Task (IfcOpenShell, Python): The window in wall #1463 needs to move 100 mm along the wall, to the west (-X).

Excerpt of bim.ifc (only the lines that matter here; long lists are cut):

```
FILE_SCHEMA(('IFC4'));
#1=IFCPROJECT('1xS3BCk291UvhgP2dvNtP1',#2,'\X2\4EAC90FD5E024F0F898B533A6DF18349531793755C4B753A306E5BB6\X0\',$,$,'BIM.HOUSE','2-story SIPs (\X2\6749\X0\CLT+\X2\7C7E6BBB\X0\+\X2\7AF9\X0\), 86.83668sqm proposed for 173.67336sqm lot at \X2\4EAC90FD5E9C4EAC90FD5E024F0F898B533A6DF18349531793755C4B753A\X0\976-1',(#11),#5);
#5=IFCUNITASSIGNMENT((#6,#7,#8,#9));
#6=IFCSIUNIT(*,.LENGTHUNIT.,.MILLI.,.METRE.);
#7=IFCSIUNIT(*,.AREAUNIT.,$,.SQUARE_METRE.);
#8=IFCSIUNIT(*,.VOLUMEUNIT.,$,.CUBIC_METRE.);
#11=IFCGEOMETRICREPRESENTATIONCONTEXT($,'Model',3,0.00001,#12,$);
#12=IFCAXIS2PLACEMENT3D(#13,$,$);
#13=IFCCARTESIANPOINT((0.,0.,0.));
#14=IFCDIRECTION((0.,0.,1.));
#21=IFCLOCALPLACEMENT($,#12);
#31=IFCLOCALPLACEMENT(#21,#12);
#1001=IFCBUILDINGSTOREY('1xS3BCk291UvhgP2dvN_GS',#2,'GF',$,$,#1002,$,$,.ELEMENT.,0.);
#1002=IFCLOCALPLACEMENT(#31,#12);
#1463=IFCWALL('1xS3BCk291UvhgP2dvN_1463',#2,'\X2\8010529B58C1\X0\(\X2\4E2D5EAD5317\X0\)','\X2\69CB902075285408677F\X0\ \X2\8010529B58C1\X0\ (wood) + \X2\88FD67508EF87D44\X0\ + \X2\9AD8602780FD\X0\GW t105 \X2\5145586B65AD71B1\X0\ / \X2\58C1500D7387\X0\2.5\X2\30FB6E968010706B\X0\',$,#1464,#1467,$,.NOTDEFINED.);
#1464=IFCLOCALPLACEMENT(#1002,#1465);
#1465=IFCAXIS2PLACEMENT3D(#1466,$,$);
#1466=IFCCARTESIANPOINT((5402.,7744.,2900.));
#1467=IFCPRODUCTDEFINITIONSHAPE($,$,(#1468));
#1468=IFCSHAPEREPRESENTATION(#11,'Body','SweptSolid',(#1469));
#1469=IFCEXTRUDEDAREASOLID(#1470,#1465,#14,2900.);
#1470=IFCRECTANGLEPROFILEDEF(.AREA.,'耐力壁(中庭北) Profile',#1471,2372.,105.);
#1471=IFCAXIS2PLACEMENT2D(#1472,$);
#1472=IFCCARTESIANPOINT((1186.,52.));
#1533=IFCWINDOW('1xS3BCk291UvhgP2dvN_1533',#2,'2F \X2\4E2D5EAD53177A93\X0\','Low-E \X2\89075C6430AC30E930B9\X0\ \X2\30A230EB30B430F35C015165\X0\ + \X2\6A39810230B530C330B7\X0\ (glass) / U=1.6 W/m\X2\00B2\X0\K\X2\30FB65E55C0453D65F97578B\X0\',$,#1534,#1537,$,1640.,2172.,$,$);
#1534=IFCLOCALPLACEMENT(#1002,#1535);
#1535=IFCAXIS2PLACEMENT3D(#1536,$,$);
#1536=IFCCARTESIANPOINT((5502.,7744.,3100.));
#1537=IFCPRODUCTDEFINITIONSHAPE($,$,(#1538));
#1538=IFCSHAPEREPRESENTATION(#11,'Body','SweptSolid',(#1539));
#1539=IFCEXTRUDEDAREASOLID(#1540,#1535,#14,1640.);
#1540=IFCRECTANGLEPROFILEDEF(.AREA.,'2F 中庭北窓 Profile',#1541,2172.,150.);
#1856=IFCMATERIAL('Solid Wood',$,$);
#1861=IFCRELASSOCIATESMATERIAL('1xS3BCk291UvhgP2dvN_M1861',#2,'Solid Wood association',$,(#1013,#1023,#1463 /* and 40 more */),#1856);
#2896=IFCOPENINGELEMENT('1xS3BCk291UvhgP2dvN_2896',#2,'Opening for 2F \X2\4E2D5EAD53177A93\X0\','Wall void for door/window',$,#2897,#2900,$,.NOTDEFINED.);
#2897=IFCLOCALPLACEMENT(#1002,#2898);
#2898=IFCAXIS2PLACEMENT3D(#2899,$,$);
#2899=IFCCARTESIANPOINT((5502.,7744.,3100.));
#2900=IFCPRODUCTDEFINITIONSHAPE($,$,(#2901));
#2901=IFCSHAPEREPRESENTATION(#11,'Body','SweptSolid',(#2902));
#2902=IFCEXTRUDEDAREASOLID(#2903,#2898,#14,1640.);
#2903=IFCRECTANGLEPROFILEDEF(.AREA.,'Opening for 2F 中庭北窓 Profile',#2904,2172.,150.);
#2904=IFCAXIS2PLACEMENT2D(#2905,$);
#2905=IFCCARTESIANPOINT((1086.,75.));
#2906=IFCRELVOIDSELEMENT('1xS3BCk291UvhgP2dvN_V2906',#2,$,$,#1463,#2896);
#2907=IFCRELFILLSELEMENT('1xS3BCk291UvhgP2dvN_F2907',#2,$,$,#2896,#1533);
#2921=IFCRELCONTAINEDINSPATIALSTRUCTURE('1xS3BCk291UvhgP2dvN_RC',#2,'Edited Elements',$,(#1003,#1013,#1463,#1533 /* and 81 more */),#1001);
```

```python
import ifcopenshell
import ifcopenshell.api.geometry
import ifcopenshell.util.placement

model = ifcopenshell.open("bim.ifc")

window = model.by_guid("1xS3BCk291UvhgP2dvN_1533")
opening = window.FillsVoids[0].RelatingOpeningElement
wall = opening.VoidsElements[0].RelatingBuildingElement

wall_matrix = ifcopenshell.util.placement.get_local_placement(wall.ObjectPlacement)
shift = wall_matrix[:3, 0] * -100.0
before = ifcopenshell.util.placement.get_local_placement(window.ObjectPlacement)[:3, 3].copy()

# The window is not placed relative to its opening, so move both.
for product in (opening, window):
    matrix = ifcopenshell.util.placement.get_local_placement(product.ObjectPlacement)
    matrix[:3, 3] += shift
    ifcopenshell.api.geometry.edit_object_placement(model, product=product, matrix=matrix, is_si=False)

after = ifcopenshell.util.placement.get_local_placement(window.ObjectPlacement)[:3, 3]
print("window moved by", (after - before).round(3) + 0.0)

model.write("bim_updated.ifc")
```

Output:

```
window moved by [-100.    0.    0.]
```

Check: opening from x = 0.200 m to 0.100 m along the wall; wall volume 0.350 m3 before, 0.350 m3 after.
